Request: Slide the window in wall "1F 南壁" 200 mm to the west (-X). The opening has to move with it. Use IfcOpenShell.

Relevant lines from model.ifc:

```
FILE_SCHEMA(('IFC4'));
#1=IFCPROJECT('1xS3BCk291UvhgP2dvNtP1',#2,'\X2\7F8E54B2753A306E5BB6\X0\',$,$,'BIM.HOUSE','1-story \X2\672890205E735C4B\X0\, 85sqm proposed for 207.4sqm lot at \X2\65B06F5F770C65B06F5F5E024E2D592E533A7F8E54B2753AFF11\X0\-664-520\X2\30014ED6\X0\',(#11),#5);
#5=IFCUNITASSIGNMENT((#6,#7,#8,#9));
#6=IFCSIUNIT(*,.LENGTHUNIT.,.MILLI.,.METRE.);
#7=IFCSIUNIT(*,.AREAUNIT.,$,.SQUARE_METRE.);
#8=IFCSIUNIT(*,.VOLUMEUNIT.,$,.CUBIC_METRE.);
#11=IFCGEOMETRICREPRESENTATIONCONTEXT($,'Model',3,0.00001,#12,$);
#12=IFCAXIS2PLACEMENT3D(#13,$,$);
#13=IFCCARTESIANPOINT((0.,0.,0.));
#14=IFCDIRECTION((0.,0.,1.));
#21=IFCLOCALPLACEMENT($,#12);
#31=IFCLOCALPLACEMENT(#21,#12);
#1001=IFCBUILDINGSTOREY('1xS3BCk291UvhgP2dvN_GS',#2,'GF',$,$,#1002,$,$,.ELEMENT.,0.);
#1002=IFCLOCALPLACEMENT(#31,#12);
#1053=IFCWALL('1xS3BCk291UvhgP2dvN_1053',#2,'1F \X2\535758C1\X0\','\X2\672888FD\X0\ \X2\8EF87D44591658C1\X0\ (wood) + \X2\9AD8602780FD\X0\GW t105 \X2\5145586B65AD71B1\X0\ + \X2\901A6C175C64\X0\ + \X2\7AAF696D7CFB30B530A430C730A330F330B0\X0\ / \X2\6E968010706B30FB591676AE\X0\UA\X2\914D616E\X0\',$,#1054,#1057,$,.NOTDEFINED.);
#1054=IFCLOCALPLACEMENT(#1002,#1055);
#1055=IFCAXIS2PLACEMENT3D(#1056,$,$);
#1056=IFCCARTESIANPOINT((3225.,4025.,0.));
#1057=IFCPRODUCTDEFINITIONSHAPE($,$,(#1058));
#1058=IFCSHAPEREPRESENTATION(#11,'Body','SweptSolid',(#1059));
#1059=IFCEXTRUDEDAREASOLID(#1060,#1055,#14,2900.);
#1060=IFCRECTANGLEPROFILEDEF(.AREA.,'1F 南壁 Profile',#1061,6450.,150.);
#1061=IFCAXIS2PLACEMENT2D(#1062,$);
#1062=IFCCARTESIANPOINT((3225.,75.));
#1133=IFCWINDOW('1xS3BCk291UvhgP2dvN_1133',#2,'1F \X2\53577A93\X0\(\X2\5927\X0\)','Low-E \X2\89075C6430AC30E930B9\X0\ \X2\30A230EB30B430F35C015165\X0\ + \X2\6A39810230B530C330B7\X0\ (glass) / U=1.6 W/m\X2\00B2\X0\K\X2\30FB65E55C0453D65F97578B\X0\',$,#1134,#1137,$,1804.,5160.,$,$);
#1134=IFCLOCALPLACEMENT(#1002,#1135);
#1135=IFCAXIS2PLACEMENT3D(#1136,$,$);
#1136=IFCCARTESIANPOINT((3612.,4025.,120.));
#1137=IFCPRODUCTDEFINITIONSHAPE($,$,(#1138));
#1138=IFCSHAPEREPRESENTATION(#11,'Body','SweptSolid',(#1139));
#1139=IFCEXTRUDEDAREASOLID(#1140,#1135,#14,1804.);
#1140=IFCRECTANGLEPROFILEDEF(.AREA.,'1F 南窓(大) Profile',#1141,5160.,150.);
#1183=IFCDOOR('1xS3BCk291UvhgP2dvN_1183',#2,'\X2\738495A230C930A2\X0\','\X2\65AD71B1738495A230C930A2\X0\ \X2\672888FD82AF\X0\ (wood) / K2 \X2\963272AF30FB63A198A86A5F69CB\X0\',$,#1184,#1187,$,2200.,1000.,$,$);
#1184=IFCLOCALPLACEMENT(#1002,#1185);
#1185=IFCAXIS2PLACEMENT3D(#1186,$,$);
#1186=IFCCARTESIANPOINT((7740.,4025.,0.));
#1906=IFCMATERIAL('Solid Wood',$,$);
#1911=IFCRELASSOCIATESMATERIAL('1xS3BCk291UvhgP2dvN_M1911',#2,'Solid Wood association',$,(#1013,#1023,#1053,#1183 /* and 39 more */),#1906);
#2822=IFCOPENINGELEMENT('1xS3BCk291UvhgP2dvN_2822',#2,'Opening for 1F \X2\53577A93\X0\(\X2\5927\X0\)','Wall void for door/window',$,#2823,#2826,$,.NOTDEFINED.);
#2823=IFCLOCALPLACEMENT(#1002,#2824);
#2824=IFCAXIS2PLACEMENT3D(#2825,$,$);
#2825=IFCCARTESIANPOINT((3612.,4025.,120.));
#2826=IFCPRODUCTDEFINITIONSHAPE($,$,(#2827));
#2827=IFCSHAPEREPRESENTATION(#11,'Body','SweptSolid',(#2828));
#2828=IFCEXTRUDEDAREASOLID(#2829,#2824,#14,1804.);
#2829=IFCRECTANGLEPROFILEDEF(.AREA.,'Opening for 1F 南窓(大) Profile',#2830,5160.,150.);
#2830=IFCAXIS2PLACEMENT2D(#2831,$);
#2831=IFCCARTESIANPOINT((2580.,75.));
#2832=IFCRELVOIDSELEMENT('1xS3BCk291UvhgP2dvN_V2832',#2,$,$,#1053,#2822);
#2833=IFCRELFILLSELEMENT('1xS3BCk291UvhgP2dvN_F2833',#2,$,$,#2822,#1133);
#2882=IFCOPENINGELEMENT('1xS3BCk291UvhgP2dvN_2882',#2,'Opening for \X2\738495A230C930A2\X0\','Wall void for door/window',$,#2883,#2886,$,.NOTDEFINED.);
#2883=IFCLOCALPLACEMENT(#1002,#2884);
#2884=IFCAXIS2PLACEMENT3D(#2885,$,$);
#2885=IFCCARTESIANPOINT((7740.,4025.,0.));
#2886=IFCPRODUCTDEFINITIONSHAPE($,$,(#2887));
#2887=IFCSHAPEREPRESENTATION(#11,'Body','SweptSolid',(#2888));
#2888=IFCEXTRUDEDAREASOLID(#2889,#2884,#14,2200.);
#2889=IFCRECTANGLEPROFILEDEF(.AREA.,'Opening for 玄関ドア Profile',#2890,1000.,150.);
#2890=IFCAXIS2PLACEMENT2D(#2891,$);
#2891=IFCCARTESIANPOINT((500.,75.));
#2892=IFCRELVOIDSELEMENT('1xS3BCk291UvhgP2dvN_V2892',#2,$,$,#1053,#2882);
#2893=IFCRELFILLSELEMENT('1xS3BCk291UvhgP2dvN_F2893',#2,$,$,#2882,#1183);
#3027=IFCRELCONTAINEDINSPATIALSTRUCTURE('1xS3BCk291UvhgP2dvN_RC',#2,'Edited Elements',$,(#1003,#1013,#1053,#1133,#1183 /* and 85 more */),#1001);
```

```python
import ifcopenshell
import ifcopenshell.api.geometry
import ifcopenshell.util.placement

model = ifcopenshell.open("model.ifc")

window = model.by_guid("1xS3BCk291UvhgP2dvN_1133")
opening = window.FillsVoids[0].RelatingOpeningElement
wall = opening.VoidsElements[0].RelatingBuildingElement

wall_matrix = ifcopenshell.util.placement.get_local_placement(wall.ObjectPlacement)
shift = wall_matrix[:3, 0] * -200.0
before = ifcopenshell.util.placement.get_local_placement(window.ObjectPlacement)[:3, 3].copy()

# The window is not placed relative to its opening, so move both.
for product in (opening, window):
    matrix = ifcopenshell.util.placement.get_local_placement(product.ObjectPlacement)
    matrix[:3, 3] += shift
    ifcopenshell.api.geometry.edit_object_placement(model, product=product, matrix=matrix, is_si=False)

after = ifcopenshell.util.placement.get_local_placement(window.ObjectPlacement)[:3, 3]
print("window moved by", (after - before).round(3) + 0.0)

model.write("model_updated.ifc")
```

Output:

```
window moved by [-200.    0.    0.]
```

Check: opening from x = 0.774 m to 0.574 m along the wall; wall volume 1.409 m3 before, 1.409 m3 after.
